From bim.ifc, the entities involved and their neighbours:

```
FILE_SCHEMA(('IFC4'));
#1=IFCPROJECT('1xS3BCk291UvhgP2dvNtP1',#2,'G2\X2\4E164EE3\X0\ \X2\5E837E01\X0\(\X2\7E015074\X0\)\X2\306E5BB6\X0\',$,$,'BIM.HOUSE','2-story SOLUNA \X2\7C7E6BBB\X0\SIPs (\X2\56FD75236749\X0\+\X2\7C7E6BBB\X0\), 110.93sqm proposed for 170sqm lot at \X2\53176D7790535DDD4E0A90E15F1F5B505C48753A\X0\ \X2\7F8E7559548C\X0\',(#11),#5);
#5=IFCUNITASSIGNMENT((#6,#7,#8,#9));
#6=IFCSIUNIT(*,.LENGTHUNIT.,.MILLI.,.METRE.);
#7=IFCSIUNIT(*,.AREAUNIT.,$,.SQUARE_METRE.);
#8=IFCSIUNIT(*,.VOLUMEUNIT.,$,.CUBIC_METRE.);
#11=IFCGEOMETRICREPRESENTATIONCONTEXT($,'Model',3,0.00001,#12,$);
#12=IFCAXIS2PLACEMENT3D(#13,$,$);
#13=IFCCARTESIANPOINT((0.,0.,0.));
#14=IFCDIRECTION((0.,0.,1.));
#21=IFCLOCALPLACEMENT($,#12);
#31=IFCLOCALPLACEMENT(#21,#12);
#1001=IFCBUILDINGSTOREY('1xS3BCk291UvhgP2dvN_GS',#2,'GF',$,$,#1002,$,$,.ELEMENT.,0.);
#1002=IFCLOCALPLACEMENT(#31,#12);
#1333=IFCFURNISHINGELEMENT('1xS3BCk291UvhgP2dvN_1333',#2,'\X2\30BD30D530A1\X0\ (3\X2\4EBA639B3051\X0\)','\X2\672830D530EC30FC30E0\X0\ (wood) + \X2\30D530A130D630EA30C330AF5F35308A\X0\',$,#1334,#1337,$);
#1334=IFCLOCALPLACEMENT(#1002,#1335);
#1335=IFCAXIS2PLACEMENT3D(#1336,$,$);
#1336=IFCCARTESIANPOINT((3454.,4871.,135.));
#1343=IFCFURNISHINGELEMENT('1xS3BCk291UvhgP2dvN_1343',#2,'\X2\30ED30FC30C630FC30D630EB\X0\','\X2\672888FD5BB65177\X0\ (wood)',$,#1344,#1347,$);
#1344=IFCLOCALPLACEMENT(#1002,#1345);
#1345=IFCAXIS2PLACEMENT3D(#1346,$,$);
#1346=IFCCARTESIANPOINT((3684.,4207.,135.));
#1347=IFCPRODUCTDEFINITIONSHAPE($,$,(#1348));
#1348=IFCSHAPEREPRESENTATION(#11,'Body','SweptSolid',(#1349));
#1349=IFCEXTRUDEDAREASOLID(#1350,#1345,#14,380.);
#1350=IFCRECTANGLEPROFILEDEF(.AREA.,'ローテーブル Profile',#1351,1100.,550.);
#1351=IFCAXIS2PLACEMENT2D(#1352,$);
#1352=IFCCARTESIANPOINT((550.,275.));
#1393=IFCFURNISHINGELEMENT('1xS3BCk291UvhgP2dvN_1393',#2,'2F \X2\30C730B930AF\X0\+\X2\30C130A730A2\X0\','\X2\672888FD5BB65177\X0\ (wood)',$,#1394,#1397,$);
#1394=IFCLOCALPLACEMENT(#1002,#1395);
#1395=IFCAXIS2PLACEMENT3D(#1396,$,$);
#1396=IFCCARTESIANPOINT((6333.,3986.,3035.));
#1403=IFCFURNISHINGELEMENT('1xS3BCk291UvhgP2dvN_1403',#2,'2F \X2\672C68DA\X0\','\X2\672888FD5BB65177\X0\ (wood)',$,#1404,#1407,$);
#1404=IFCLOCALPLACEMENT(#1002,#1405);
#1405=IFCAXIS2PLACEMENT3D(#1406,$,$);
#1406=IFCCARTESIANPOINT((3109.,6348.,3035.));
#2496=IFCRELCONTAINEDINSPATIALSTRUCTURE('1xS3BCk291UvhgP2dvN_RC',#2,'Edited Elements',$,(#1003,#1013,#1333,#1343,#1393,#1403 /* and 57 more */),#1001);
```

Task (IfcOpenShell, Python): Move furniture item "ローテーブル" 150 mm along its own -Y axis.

```python
import ifcopenshell
import ifcopenshell.api.geometry
import ifcopenshell.util.placement
import ifcopenshell.util.unit

model = ifcopenshell.open("bim.ifc")
unit_scale = ifcopenshell.util.unit.calculate_unit_scale(model)

item = model.by_guid("1xS3BCk291UvhgP2dvN_1343")
matrix = ifcopenshell.util.placement.get_local_placement(item.ObjectPlacement)
matrix[:3, 3] -= matrix[:3, 1] * 0.15 / unit_scale
ifcopenshell.api.geometry.edit_object_placement(model, product=item, matrix=matrix, is_si=False)

print(ifcopenshell.util.placement.get_local_placement(item.ObjectPlacement).round(3) + 0.0)

model.write("bim_rev.ifc")
```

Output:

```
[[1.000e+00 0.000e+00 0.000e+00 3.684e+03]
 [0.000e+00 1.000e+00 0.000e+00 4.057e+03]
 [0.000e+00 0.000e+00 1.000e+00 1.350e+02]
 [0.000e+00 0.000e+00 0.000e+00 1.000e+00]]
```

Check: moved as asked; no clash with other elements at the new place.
